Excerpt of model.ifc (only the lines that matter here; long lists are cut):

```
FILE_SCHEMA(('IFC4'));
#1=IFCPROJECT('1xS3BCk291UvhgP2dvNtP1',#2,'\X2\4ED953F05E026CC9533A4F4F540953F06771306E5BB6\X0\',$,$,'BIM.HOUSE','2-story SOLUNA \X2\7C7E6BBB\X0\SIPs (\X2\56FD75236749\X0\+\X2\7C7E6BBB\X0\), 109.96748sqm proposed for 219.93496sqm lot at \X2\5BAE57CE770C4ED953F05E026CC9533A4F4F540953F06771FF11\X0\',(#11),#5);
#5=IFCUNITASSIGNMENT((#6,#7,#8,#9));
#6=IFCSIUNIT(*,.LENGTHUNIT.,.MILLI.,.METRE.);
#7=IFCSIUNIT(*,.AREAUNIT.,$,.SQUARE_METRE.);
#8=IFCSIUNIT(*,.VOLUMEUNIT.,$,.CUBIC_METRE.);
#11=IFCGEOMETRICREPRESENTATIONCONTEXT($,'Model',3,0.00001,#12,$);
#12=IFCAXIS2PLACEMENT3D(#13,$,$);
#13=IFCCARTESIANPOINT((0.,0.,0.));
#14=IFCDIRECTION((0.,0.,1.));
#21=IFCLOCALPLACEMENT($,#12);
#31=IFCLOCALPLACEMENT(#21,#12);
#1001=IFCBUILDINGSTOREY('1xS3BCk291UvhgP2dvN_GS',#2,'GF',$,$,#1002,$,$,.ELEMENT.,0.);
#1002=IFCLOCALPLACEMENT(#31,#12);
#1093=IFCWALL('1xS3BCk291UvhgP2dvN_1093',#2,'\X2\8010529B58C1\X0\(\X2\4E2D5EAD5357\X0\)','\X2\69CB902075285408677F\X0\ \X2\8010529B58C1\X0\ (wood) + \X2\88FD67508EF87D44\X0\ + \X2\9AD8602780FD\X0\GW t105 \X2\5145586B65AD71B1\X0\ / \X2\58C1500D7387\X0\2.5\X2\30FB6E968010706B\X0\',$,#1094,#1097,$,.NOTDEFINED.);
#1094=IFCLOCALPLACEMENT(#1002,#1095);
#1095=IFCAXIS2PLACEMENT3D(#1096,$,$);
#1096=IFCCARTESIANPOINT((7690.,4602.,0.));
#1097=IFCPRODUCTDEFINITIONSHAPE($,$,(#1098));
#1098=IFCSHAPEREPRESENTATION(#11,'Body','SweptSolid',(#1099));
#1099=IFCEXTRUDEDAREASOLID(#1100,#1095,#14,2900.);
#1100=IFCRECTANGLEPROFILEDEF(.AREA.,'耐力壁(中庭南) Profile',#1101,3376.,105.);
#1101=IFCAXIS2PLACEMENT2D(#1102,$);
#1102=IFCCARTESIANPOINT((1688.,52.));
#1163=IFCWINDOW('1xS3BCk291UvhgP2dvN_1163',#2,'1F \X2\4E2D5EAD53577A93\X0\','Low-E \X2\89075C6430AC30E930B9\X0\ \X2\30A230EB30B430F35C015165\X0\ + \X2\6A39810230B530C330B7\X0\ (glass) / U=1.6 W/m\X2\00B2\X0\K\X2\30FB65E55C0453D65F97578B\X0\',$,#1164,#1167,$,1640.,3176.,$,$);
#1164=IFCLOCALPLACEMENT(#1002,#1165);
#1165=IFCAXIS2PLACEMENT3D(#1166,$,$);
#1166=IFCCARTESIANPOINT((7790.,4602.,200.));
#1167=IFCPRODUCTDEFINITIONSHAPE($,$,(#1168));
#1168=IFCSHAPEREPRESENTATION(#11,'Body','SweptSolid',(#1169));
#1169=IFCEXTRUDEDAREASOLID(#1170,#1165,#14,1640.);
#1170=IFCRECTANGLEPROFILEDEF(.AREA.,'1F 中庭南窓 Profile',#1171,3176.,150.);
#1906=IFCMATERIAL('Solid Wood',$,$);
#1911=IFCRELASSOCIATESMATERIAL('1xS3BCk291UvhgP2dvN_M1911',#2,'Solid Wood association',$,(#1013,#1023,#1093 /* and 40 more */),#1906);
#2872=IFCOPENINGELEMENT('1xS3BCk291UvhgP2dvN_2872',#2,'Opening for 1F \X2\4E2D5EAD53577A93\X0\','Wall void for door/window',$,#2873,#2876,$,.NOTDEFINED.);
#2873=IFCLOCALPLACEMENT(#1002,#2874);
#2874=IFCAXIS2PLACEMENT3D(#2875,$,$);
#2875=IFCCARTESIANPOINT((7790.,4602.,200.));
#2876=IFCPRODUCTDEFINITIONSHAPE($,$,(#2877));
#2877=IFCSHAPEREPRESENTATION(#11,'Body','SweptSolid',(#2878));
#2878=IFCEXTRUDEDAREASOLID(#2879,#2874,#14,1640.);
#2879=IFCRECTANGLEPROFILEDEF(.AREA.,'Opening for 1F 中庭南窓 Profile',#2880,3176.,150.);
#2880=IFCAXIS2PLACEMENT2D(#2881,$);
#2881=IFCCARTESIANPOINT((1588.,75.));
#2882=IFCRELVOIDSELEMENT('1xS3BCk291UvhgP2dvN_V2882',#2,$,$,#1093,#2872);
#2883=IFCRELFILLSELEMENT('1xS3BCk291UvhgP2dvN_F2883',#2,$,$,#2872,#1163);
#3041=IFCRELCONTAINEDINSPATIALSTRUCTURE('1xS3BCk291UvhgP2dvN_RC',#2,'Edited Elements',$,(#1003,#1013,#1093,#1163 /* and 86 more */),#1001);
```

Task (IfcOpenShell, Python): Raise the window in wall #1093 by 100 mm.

```python
import numpy as np
import ifcopenshell
import ifcopenshell.api.geometry
import ifcopenshell.util.placement
import ifcopenshell.util.unit

model = ifcopenshell.open("model.ifc")
unit_scale = ifcopenshell.util.unit.calculate_unit_scale(model)

window = model.by_guid("1xS3BCk291UvhgP2dvN_1163")
opening = window.FillsVoids[0].RelatingOpeningElement
dz = 0.1 / unit_scale

shift = np.array([0.0, 0.0, dz])
# The window is not placed relative to its opening, so move both.
for product in (opening, window):
    matrix = ifcopenshell.util.placement.get_local_placement(product.ObjectPlacement)
    matrix[:3, 3] += shift
    ifcopenshell.api.geometry.edit_object_placement(model, product=product, matrix=matrix, is_si=False)

print(f"moved by {dz * unit_scale:+.3f} m")

model.write("model-out.ifc")
```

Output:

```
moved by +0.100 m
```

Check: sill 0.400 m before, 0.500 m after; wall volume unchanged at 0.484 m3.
